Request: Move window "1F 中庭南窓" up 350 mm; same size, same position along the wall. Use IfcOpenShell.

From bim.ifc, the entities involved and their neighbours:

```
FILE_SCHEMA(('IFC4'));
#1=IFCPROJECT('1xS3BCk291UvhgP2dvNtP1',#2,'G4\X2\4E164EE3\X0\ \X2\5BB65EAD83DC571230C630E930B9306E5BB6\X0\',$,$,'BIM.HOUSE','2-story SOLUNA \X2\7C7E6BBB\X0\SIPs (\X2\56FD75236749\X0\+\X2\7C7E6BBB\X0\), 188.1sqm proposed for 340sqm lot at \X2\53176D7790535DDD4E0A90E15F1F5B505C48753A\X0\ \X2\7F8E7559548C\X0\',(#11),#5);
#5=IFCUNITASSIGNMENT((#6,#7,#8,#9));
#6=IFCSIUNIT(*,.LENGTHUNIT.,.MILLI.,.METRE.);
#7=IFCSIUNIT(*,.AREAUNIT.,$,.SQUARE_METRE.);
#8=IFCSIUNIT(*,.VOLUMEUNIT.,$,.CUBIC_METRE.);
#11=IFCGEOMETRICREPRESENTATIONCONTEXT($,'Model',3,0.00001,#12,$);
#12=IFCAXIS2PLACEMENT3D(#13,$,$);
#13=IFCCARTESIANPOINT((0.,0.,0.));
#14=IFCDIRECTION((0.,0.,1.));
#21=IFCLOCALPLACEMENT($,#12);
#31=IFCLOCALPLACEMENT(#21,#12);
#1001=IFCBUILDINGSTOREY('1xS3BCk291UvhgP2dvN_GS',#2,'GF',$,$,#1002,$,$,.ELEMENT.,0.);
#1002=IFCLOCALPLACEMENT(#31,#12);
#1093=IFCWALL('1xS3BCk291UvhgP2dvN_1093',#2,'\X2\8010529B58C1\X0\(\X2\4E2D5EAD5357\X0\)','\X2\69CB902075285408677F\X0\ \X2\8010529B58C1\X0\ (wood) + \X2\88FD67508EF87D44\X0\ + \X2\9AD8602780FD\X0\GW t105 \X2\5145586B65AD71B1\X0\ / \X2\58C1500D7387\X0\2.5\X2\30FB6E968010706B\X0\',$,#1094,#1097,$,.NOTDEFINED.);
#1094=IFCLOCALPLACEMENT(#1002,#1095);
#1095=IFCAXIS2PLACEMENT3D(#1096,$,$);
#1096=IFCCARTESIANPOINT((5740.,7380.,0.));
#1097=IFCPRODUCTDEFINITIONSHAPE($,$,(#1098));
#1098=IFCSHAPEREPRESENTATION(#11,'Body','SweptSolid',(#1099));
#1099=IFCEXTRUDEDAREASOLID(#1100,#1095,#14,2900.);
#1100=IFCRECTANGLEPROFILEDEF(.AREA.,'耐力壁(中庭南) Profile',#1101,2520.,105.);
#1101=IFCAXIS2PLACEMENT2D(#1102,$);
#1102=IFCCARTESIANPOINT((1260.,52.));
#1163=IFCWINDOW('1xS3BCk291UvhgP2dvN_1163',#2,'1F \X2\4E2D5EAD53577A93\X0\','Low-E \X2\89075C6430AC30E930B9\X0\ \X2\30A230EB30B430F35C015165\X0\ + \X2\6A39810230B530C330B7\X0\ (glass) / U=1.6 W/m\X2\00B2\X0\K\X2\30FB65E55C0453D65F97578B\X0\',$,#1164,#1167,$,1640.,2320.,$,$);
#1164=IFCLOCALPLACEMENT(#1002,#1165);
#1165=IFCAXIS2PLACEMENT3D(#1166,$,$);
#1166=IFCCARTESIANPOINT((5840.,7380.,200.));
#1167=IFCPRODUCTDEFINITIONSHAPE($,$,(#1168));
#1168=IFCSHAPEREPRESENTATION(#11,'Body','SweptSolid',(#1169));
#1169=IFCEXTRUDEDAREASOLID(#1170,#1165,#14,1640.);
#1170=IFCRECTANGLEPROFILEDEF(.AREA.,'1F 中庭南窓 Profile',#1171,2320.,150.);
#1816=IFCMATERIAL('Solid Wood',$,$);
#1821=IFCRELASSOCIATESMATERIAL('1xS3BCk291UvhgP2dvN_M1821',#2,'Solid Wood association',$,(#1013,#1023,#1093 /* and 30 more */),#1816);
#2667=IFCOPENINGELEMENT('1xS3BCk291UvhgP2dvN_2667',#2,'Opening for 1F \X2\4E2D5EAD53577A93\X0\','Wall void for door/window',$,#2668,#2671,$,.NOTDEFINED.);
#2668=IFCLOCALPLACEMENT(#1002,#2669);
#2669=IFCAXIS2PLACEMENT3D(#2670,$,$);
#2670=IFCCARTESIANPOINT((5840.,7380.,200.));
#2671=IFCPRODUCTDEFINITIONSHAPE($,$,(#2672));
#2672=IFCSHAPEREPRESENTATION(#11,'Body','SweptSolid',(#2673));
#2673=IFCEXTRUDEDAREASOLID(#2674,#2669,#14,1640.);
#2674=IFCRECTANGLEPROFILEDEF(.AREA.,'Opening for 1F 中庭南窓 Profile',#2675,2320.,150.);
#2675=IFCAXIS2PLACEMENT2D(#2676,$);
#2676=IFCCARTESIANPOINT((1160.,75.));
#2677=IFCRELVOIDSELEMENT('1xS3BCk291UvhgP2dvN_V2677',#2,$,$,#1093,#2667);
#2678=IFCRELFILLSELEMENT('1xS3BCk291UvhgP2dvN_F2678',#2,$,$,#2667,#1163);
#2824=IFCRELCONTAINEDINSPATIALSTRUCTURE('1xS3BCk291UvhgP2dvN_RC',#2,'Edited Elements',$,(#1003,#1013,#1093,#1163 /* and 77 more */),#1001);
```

```python
import numpy as np
import ifcopenshell
import ifcopenshell.api.geometry
import ifcopenshell.util.placement
import ifcopenshell.util.unit

model = ifcopenshell.open("bim.ifc")
unit_scale = ifcopenshell.util.unit.calculate_unit_scale(model)

window = model.by_id(1163)
opening = window.FillsVoids[0].RelatingOpeningElement
dz = 0.35 / unit_scale

shift = np.array([0.0, 0.0, dz])
# The window is not placed relative to its opening, so move both.
for product in (opening, window):
    matrix = ifcopenshell.util.placement.get_local_placement(product.ObjectPlacement)
    matrix[:3, 3] += shift
    ifcopenshell.api.geometry.edit_object_placement(model, product=product, matrix=matrix, is_si=False)

print(f"moved by {dz * unit_scale:+.3f} m")

model.write("bim-out.ifc")
```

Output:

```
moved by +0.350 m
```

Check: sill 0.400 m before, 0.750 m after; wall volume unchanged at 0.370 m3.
